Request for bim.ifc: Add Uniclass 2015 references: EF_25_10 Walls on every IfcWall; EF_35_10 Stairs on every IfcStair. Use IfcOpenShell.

First a look at what the model holds.

```python
import ifcopenshell

model = ifcopenshell.open("bim.ifc")
print(model.schema)
print("classifications:", [c.Name for c in model.by_type("IfcClassification")])
for ifc_class in ("IfcDoor", "IfcRoof", "IfcStair", "IfcWall", "IfcWindow"):
    print(ifc_class, len(model.by_type(ifc_class)))
```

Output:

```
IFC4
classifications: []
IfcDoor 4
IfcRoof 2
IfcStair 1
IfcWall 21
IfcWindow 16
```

```python
import ifcopenshell
import ifcopenshell.api.classification

model = ifcopenshell.open("bim.ifc")

system = ifcopenshell.api.classification.add_classification(model, classification="Uniclass 2015")

codes = {
    "IfcWall": ("EF_25_10", "Walls"),
    "IfcStair": ("EF_35_10", "Stairs"),
}
for ifc_class, (code, name) in codes.items():
    products = model.by_type(ifc_class)
    ifcopenshell.api.classification.add_reference(
        model, products=products, classification=system, identification=code, name=name
    )
    print(code, len(products))

model.write("bim_rev.ifc")
```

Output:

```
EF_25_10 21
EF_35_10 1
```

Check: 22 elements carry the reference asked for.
